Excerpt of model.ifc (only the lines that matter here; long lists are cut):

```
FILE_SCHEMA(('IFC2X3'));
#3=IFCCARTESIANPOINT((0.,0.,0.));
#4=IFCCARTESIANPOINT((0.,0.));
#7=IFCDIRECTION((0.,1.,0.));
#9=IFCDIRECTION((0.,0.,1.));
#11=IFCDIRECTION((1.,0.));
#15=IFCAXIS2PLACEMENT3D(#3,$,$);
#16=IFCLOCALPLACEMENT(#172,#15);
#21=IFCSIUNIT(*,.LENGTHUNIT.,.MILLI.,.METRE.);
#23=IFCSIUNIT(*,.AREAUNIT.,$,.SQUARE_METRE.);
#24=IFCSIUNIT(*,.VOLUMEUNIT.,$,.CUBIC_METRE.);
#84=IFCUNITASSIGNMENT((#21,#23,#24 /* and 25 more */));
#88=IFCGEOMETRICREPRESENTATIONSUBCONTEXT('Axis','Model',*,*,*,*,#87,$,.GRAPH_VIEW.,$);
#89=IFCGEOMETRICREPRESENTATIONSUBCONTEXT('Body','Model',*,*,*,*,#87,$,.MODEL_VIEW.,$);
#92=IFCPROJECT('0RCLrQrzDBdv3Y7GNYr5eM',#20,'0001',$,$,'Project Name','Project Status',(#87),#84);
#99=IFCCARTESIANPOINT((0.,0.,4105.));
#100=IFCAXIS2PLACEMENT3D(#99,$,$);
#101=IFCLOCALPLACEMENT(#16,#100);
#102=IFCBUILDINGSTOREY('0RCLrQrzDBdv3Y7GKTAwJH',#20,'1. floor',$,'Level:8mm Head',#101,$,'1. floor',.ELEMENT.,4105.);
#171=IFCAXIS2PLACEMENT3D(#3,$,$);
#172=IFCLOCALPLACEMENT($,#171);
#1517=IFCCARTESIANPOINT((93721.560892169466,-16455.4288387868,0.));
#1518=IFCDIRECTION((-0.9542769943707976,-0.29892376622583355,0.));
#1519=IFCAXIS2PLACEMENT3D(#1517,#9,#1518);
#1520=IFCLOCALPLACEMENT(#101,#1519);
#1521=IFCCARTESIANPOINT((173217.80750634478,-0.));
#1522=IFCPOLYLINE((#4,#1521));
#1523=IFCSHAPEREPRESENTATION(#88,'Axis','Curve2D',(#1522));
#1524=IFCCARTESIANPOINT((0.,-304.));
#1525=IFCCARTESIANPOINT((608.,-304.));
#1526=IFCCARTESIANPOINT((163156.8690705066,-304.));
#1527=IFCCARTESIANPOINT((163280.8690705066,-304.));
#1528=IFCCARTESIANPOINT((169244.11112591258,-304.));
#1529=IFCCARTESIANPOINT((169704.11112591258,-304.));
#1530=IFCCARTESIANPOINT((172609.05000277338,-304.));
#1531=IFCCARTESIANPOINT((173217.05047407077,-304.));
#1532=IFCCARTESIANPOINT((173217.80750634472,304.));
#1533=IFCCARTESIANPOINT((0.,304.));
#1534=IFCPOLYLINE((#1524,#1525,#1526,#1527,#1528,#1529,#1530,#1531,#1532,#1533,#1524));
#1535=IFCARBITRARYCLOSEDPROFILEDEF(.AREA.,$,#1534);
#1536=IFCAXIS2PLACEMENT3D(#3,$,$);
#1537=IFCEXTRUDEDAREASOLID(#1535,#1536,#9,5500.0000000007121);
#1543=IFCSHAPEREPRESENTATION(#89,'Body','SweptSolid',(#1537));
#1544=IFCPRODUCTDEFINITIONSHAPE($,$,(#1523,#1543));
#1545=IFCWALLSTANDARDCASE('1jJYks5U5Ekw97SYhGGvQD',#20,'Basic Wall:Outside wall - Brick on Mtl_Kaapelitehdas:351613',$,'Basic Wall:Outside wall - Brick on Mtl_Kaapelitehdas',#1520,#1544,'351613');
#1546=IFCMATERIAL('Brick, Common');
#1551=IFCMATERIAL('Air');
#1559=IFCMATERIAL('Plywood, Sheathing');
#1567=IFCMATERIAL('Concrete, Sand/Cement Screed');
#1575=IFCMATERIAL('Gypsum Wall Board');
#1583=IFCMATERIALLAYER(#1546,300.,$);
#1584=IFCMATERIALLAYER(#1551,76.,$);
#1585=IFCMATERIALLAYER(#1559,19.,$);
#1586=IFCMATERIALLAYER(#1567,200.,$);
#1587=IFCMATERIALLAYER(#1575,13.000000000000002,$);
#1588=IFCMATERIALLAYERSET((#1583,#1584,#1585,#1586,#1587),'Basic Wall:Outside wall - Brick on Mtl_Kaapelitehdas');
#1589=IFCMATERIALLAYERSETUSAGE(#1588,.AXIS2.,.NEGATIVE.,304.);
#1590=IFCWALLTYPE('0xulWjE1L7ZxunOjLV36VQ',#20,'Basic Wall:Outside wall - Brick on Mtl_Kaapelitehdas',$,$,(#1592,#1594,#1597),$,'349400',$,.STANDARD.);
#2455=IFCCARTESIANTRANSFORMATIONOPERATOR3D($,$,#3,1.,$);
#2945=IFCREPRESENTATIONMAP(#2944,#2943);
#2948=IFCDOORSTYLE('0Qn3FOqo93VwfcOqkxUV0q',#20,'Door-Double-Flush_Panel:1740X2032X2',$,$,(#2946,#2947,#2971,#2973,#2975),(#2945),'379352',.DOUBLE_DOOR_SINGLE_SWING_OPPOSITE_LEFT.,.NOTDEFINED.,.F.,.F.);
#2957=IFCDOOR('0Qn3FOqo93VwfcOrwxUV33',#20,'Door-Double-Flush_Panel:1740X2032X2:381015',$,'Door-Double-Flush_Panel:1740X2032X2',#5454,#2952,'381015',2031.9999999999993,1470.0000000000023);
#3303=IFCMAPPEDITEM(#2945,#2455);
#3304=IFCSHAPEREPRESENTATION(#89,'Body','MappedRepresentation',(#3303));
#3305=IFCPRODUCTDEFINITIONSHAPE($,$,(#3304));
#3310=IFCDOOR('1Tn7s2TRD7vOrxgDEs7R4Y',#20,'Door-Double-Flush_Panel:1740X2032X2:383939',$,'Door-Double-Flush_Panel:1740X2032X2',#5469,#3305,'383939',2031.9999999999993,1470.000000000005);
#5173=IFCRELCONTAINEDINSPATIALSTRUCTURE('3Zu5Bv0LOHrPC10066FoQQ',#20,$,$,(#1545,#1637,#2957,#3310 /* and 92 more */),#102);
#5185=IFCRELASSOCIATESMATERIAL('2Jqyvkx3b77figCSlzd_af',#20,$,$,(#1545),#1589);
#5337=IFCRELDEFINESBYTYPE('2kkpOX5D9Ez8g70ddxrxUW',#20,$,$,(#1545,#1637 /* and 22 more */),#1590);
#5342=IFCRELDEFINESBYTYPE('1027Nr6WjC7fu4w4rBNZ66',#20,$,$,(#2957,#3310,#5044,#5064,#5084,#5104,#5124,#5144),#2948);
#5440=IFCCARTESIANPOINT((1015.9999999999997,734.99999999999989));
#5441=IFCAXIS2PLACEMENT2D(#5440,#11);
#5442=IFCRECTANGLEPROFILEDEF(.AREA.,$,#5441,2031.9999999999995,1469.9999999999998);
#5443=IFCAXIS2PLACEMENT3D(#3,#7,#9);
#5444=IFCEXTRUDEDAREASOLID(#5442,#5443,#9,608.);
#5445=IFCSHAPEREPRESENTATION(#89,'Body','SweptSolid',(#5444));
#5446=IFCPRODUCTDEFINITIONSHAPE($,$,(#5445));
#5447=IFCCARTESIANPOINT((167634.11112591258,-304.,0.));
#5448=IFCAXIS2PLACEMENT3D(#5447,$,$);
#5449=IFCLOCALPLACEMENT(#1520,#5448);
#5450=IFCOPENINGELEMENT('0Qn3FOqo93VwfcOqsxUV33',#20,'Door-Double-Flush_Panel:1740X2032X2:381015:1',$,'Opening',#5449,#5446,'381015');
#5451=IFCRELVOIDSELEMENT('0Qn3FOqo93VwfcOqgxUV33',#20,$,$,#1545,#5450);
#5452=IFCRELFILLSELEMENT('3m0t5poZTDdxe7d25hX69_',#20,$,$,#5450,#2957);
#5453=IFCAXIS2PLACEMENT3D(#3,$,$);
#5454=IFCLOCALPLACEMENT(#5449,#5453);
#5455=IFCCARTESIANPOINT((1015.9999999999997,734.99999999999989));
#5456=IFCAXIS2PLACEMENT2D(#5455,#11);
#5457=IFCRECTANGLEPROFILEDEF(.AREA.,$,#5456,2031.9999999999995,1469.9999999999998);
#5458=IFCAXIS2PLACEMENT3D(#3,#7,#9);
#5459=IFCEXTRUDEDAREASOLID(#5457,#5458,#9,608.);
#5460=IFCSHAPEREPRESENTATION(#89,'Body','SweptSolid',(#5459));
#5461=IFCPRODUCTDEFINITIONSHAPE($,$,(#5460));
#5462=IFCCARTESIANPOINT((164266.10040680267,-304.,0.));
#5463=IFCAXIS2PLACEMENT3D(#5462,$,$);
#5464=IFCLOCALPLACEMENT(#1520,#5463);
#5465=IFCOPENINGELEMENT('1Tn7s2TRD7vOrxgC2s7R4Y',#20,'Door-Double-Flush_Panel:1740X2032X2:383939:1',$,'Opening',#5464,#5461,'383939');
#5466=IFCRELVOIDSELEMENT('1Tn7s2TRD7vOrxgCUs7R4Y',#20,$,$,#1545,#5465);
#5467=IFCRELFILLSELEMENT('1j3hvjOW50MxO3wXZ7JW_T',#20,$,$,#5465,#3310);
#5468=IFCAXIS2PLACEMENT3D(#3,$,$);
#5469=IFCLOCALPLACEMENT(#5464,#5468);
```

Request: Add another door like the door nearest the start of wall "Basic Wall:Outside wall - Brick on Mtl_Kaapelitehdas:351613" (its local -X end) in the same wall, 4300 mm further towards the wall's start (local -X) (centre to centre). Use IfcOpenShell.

```python
import ifcopenshell
import ifcopenshell.api.feature
import ifcopenshell.api.geometry
import ifcopenshell.api.root
import ifcopenshell.geom
import ifcopenshell.util.element
import ifcopenshell.util.placement
import ifcopenshell.util.shape

model = ifcopenshell.open("model.ifc")
settings = ifcopenshell.geom.settings()


def volume(element):
    """Net volume in cubic metres, openings subtracted."""
    shape = ifcopenshell.geom.create_shape(settings, element)
    return ifcopenshell.util.shape.get_volume(shape.geometry)


def reuse_history(source, copy):
    """copy_class also copies each property set's owner history, people and application; keep the originals."""
    for rel in copy.IsDefinedBy:
        if rel.is_a("IfcRelDefinesByProperties") and (history := rel.RelatingPropertyDefinition.OwnerHistory):
            rel.RelatingPropertyDefinition.OwnerHistory = source.OwnerHistory
            ifcopenshell.util.element.remove_deep2(model, history)


door = model.by_id(3310)
opening = door.FillsVoids[0].RelatingOpeningElement
wall = opening.VoidsElements[0].RelatingBuildingElement
before = volume(wall)
shift = ifcopenshell.util.placement.get_local_placement(wall.ObjectPlacement)[:3, 0] * -4300.0

# copy_class copies the void relationship, type, container and properties, but no geometry.
new_opening = ifcopenshell.api.root.copy_class(model, product=opening)
new_opening.Representation = ifcopenshell.util.element.copy_deep(
    model, opening.Representation, exclude=["IfcGeometricRepresentationContext", "IfcRepresentationMap"]
)
new_opening.Name = "Door-Double-Flush_Panel:1740X2032X2"
new_opening.Tag = None
new_door = ifcopenshell.api.root.copy_class(model, product=door)
new_door.Representation = ifcopenshell.util.element.copy_deep(
    model, door.Representation, exclude=["IfcGeometricRepresentationContext", "IfcRepresentationMap"]
)
new_door.Name = "Door-Double-Flush_Panel:1740X2032X2"
new_door.Tag = None
reuse_history(door, new_door)
fills = ifcopenshell.api.feature.add_filling(model, opening=new_opening, element=new_door)
fills.OwnerHistory = new_door.OwnerHistory  # required in IFC2X3

for old, new in ((opening, new_opening), (door, new_door)):
    matrix = ifcopenshell.util.placement.get_local_placement(old.ObjectPlacement)
    matrix[:3, 3] += shift
    ifcopenshell.api.geometry.edit_object_placement(model, product=new, matrix=matrix, is_si=False)

after = volume(wall)

print(f"wall volume {before:.3f} -> {after:.3f} m3")

model.write("model_v2.ifc")
```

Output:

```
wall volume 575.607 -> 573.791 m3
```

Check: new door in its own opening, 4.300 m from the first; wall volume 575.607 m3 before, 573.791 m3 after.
